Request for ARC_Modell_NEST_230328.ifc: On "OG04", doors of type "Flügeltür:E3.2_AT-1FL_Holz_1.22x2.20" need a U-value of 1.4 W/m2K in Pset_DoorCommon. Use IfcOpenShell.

First a look at what the model holds.

```python
import ifcopenshell
import ifcopenshell.util.element

model = ifcopenshell.open("ARC_Modell_NEST_230328.ifc")
print(model.schema)
storey = next(s for s in model.by_type("IfcBuildingStorey") if s.Name == "OG04")
doors = [e for e in ifcopenshell.util.element.get_decomposition(storey) if e.is_a("IfcDoor")]
seen = {}
for e in doors:
    element_type = ifcopenshell.util.element.get_type(e)
    key = (element_type.Name if element_type != e and element_type else None, ifcopenshell.util.element.get_pset(e, "Pset_DoorCommon", "ThermalTransmittance"))
    seen[key] = seen.get(key, 0) + 1
for (name, value), count in sorted(seen.items(), key=str):
    print(count, "x", name, "|", value)
```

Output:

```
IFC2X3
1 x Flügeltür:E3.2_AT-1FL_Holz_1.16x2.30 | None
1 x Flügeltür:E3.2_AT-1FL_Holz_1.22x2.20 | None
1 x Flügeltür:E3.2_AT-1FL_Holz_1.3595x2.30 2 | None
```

```python
import ifcopenshell
import ifcopenshell.api.pset
import ifcopenshell.util.element

model = ifcopenshell.open("ARC_Modell_NEST_230328.ifc")

storey = next(s for s in model.by_type("IfcBuildingStorey") if s.Name == "OG04")
doors = [e for e in ifcopenshell.util.element.get_decomposition(storey) if e.is_a("IfcDoor")]

count = 0
for e in doors:
    element_type = ifcopenshell.util.element.get_type(e)
    if element_type in (None, e) or element_type.Name != "Flügeltür:E3.2_AT-1FL_Holz_1.22x2.20":
        continue
    # add_pset returns the element's existing set when there is one.
    pset = ifcopenshell.api.pset.add_pset(model, product=e, name="Pset_DoorCommon")
    ifcopenshell.api.pset.edit_pset(model, pset=pset, properties={"ThermalTransmittance": 1.4})
    count += 1

print(count, "doors updated")

model.write("ARC_Modell_NEST_230328_rev.ifc")
```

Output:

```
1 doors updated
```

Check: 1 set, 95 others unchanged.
